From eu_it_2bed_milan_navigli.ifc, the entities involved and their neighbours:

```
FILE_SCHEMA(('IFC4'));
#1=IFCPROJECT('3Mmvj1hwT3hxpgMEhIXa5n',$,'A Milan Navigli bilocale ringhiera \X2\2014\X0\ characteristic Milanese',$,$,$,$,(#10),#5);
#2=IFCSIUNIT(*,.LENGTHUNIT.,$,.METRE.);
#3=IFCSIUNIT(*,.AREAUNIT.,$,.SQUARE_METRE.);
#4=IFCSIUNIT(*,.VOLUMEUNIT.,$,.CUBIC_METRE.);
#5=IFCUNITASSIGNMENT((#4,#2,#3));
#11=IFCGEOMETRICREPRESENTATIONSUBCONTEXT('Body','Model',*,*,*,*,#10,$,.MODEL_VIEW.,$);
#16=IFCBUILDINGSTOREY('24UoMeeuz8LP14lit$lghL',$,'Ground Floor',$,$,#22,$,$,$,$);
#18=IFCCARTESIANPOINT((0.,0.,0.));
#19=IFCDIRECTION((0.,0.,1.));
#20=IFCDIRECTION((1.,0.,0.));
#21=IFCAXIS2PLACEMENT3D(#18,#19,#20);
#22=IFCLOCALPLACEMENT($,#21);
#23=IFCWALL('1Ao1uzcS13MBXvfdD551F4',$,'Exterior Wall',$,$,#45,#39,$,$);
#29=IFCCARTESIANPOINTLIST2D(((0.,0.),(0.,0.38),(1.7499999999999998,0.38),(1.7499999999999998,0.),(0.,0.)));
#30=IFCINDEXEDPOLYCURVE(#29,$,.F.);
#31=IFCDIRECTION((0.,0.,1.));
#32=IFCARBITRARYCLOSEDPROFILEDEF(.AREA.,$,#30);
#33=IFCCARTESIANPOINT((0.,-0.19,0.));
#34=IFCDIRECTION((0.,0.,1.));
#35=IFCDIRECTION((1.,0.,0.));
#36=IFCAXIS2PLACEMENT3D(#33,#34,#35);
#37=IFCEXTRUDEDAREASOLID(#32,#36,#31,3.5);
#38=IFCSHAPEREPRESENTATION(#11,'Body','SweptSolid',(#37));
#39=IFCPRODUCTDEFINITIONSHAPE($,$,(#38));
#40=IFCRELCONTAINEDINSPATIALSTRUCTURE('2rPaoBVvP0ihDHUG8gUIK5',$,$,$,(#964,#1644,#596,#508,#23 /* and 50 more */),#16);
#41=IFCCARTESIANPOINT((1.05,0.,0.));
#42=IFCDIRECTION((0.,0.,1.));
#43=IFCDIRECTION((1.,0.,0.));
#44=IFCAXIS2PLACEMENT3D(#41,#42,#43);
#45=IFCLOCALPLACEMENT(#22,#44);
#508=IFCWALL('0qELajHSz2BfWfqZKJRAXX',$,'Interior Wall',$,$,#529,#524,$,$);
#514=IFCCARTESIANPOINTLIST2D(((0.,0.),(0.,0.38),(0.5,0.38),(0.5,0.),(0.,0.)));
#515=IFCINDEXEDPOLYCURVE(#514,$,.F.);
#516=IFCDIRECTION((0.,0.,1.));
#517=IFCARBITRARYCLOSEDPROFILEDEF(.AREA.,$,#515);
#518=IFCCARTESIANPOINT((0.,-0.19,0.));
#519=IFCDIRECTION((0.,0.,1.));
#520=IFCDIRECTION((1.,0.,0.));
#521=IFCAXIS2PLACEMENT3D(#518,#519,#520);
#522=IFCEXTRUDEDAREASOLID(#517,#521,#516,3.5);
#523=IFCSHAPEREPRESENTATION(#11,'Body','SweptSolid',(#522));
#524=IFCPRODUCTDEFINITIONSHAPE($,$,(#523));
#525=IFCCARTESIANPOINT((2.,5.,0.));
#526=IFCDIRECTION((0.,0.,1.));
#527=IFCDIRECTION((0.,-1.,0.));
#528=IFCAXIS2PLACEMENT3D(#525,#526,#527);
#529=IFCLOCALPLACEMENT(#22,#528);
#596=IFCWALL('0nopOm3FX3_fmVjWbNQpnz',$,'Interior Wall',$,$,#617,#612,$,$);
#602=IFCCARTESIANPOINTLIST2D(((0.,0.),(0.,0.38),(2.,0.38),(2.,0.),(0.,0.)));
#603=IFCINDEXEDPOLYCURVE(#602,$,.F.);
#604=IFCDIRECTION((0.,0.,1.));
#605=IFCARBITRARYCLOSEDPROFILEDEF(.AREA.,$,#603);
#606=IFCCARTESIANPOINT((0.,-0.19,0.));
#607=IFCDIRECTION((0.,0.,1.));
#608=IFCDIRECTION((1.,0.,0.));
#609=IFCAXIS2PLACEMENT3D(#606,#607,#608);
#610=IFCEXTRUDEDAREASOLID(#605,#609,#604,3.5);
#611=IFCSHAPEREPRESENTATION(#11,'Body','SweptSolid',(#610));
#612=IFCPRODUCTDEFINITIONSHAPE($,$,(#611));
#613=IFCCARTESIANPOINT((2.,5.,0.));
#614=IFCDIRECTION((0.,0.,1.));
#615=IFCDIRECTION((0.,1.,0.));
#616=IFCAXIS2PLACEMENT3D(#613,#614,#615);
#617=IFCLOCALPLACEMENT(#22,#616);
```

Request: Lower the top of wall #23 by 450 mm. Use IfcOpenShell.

```python
import ifcopenshell
import ifcopenshell.geom
import ifcopenshell.util.representation
import ifcopenshell.util.shape
import ifcopenshell.util.unit

model = ifcopenshell.open("eu_it_2bed_milan_navigli.ifc")
unit_scale = ifcopenshell.util.unit.calculate_unit_scale(model)
settings = ifcopenshell.geom.settings()


def volume(element):
    """Net volume in cubic metres, openings subtracted."""
    shape = ifcopenshell.geom.create_shape(settings, element)
    return ifcopenshell.util.shape.get_volume(shape.geometry)


wall = model.by_guid("1Ao1uzcS13MBXvfdD551F4")
before = volume(wall)

body = ifcopenshell.util.representation.get_representation(wall, "Model", "Body")
solid = body.Items[0]
old_height = solid.Depth
solid.Depth -= 0.45 / unit_scale
after = volume(wall)

print(f"height {old_height:g} -> {solid.Depth:g}, volume {before:.3f} -> {after:.3f} m3")

model.write("eu_it_2bed_milan_navigli_edited.ifc")
```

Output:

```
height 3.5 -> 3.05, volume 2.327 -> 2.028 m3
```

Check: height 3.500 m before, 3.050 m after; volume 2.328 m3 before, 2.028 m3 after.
